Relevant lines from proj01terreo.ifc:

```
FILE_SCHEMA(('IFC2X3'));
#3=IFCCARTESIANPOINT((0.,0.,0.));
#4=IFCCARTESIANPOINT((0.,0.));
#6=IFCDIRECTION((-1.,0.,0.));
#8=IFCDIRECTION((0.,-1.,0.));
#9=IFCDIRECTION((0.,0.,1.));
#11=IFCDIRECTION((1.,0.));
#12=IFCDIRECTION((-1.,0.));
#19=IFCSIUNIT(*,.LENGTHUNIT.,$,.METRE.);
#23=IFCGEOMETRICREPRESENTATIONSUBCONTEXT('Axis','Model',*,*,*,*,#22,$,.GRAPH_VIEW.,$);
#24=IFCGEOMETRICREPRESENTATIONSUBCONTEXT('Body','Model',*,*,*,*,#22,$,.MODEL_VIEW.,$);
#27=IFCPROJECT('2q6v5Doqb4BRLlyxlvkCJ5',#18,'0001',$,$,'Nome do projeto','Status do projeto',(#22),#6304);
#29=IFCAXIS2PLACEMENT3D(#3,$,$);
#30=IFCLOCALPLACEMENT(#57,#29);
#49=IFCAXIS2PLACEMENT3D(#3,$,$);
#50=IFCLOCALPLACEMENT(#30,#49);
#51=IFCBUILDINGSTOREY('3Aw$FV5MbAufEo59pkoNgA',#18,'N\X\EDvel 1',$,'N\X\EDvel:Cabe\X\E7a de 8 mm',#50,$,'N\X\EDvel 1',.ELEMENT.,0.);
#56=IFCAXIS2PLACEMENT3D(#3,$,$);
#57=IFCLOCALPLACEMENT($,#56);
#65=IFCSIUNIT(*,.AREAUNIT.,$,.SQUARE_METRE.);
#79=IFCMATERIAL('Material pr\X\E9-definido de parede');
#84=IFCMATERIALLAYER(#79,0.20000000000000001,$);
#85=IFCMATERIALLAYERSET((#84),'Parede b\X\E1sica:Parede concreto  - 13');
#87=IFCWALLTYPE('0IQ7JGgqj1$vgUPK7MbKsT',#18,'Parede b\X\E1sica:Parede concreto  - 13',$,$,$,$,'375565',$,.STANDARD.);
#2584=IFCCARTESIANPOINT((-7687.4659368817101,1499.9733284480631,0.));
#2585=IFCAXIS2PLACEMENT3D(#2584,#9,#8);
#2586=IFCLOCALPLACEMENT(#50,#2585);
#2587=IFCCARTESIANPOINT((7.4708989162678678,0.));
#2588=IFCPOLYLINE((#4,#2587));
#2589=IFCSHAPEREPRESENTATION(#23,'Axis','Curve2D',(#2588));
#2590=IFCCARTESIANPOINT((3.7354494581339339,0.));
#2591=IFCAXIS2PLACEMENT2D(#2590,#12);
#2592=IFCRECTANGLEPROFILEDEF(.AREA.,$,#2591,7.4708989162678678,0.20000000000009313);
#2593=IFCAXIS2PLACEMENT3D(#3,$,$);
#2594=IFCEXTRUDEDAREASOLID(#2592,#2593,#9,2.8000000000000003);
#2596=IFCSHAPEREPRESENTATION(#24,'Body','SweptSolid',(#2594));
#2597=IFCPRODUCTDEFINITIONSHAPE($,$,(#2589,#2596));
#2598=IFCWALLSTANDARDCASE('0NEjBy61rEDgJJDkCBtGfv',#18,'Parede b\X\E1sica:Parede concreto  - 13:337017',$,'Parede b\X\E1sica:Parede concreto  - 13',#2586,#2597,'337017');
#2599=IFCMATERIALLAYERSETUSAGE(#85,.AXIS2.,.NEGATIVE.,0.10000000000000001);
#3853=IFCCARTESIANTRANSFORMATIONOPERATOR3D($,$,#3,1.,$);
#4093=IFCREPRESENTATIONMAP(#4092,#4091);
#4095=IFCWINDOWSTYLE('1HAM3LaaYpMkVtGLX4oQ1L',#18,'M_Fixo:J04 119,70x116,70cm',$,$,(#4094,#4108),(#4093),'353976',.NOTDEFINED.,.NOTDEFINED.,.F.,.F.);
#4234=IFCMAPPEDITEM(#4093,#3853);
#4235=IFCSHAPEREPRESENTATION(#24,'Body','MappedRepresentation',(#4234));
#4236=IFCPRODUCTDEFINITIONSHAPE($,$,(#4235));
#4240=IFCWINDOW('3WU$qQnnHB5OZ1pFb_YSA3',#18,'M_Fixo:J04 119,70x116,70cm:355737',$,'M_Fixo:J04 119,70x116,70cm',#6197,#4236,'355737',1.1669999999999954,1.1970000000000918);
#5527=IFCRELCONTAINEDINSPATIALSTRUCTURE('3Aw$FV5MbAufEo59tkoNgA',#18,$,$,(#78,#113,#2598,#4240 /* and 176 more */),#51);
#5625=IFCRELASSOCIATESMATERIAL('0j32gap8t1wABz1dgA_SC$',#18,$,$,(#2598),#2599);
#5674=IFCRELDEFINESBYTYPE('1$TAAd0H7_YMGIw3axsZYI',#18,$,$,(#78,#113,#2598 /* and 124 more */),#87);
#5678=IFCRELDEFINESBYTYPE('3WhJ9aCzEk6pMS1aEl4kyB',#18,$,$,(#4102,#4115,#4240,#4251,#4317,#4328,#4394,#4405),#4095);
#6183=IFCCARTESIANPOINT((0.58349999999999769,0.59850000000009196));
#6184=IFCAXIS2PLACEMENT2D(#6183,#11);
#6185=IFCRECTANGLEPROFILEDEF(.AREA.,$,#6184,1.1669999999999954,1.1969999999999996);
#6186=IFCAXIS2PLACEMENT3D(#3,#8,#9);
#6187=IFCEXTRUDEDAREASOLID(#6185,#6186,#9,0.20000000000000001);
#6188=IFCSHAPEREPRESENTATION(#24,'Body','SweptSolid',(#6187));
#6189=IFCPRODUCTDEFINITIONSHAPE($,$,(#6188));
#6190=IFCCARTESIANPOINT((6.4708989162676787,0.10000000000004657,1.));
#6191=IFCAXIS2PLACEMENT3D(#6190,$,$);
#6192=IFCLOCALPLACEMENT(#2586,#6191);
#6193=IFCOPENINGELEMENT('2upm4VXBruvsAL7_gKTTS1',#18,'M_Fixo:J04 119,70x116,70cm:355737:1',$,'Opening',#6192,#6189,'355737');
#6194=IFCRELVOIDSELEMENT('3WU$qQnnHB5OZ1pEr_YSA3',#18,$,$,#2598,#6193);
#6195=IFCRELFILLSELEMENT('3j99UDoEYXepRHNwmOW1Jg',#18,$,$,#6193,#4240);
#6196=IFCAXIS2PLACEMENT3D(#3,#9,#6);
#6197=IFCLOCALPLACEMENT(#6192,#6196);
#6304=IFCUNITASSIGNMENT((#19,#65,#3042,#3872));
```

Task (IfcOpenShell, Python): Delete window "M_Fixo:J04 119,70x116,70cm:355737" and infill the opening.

```python
import ifcopenshell
import ifcopenshell.api.feature
import ifcopenshell.api.root
import ifcopenshell.geom
import ifcopenshell.util.shape

model = ifcopenshell.open("proj01terreo.ifc")
settings = ifcopenshell.geom.settings()


def volume(element):
    """Net volume in cubic metres, openings subtracted."""
    shape = ifcopenshell.geom.create_shape(settings, element)
    return ifcopenshell.util.shape.get_volume(shape.geometry)


window = model.by_guid("3WU$qQnnHB5OZ1pFb_YSA3")
opening = window.FillsVoids[0].RelatingOpeningElement
wall = opening.VoidsElements[0].RelatingBuildingElement
before = volume(wall)

ifcopenshell.api.root.remove_product(model, product=window)
ifcopenshell.api.feature.remove_feature(model, feature=opening)

after = volume(wall)

print(f"wall volume {before:.3f} -> {after:.3f} m3")

model.write("proj01terreo_updated.ifc")
```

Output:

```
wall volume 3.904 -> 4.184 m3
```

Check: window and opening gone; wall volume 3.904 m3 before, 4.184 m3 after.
